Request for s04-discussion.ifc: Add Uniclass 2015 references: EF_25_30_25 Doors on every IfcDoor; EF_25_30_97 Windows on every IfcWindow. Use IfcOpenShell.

First a look at what the model holds.

```python
import ifcopenshell

model = ifcopenshell.open("s04-discussion.ifc")
print(model.schema)
print("classifications:", [c.Name for c in model.by_type("IfcClassification")])
for ifc_class in ("IfcDoor", "IfcRoof", "IfcStair", "IfcWall", "IfcWindow"):
    print(ifc_class, len(model.by_type(ifc_class)))
```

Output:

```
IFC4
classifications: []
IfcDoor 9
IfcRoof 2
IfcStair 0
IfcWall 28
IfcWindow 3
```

```python
import ifcopenshell
import ifcopenshell.api.classification

model = ifcopenshell.open("s04-discussion.ifc")

system = ifcopenshell.api.classification.add_classification(model, classification="Uniclass 2015")

codes = {
    "IfcDoor": ("EF_25_30_25", "Doors"),
    "IfcWindow": ("EF_25_30_97", "Windows"),
}
for ifc_class, (code, name) in codes.items():
    products = model.by_type(ifc_class)
    ifcopenshell.api.classification.add_reference(
        model, products=products, classification=system, identification=code, name=name
    )
    print(code, len(products))

model.write("s04-discussion_rev.ifc")
```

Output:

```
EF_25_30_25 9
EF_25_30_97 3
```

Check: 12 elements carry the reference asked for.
